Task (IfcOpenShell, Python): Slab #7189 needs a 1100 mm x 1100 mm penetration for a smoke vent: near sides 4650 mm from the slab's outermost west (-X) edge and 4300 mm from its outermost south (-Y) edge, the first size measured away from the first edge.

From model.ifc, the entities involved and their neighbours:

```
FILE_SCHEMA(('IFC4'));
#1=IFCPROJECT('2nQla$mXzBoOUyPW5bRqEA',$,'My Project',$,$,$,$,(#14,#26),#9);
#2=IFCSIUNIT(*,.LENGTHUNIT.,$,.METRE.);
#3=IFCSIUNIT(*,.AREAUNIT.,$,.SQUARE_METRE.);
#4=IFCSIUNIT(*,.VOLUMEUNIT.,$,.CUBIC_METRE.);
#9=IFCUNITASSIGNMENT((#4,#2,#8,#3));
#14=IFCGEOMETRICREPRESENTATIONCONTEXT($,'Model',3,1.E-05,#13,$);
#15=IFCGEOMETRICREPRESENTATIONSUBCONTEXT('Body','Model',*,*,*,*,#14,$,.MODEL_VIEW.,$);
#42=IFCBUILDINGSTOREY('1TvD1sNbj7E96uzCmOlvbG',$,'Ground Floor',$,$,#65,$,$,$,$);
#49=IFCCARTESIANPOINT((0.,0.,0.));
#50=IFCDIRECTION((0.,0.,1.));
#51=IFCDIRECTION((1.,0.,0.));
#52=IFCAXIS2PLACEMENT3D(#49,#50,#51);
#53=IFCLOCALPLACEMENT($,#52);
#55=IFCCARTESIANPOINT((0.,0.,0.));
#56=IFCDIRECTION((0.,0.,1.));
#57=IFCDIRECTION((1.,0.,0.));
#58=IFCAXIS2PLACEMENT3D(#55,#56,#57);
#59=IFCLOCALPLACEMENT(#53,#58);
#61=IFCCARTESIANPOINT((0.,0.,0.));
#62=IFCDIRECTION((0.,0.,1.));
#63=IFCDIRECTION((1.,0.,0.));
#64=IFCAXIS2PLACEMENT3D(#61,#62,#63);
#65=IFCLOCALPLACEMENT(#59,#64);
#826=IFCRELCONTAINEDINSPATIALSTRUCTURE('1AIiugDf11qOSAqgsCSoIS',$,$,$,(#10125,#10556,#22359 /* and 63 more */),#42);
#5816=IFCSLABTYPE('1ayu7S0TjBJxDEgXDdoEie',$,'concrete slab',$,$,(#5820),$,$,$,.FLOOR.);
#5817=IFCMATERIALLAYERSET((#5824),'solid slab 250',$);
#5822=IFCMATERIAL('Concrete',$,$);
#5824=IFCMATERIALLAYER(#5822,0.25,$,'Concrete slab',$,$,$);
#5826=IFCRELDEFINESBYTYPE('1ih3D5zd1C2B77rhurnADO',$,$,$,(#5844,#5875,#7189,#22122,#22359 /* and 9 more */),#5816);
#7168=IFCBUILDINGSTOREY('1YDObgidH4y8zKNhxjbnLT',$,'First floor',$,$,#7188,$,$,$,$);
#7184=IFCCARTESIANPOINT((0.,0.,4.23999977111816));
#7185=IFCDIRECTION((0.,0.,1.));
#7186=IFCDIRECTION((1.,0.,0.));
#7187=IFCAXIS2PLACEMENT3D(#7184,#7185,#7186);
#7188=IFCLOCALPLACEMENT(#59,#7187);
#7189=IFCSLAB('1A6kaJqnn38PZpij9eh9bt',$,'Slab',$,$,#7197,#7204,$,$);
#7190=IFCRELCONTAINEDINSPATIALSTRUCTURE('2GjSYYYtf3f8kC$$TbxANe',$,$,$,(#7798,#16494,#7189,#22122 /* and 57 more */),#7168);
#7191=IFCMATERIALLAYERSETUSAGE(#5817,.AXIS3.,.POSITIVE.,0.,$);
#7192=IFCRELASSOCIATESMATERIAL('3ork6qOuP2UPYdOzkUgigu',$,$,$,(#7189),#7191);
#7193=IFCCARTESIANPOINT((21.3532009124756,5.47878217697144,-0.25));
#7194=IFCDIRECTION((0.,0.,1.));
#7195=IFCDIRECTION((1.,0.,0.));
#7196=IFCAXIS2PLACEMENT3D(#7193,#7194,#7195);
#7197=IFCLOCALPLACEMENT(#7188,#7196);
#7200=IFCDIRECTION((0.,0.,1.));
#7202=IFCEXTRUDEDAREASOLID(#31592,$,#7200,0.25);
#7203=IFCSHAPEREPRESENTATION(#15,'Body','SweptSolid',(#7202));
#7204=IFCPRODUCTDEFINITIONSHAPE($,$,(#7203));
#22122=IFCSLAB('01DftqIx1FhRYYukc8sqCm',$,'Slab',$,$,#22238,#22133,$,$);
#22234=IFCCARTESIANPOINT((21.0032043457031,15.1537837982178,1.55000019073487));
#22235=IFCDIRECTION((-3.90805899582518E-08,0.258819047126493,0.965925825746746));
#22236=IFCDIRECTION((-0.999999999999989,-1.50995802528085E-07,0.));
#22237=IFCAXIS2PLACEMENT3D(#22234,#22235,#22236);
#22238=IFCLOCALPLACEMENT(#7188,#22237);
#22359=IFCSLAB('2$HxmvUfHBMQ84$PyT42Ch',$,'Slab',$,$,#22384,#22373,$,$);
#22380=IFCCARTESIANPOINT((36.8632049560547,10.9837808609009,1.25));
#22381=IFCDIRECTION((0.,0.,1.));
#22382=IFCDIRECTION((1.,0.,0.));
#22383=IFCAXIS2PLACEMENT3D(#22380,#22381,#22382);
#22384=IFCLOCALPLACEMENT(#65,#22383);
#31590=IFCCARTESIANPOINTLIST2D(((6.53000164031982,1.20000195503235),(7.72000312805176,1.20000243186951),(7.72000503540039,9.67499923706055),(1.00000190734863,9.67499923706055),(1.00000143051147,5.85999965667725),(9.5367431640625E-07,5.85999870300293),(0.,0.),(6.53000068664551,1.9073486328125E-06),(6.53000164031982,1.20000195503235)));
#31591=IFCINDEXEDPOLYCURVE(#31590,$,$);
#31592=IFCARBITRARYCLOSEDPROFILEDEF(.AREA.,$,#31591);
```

```python
import numpy as np
import ifcopenshell
import ifcopenshell.api.feature
import ifcopenshell.api.geometry
import ifcopenshell.api.root
import ifcopenshell.geom
import ifcopenshell.util.placement
import ifcopenshell.util.representation
import ifcopenshell.util.shape
import ifcopenshell.util.unit

model = ifcopenshell.open("model.ifc")
unit_scale = ifcopenshell.util.unit.calculate_unit_scale(model)
settings = ifcopenshell.geom.settings()


def volume(element):
    """Net volume in cubic metres, openings subtracted."""
    shape = ifcopenshell.geom.create_shape(settings, element)
    return ifcopenshell.util.shape.get_volume(shape.geometry)


slab = model.by_id(7189)
before = volume(slab)

# Extent in the slab's own axes, in metres. The edges named are its -X and -Y sides.
slab_shape = ifcopenshell.geom.create_shape(settings, slab)
vertices = ifcopenshell.util.shape.get_vertices(slab_shape.geometry)
x_min, y_min, bottom = vertices.min(axis=0)
top = vertices[:, 2].max()

opening = ifcopenshell.api.root.create_entity(model, ifc_class="IfcOpeningElement", name="Smoke vent opening", predefined_type="OPENING")
context = ifcopenshell.util.representation.get_context(model, "Model", "Body", "MODEL_VIEW")
width, depth = 1.1, 1.1
outline = [(0.0, 0.0), (width, 0.0), (width, depth), (0.0, depth), (0.0, 0.0)]
# Overshoot both faces by 50 mm so the cut is clean.
shape = ifcopenshell.api.geometry.add_slab_representation(
    model, context=context, depth=top - bottom + 0.1, polyline=outline
)
ifcopenshell.api.geometry.assign_representation(model, product=opening, representation=shape)

matrix = ifcopenshell.util.placement.get_local_placement(slab.ObjectPlacement)
matrix[:, 3] = matrix @ np.append(np.array([x_min + 4.65, y_min + 4.3, bottom - 0.05]) / unit_scale, 1.0)
ifcopenshell.api.geometry.edit_object_placement(model, product=opening, matrix=matrix, is_si=False)
ifcopenshell.api.feature.add_feature(model, feature=opening, element=slab)

after = volume(slab)

print(f"slab volume {before:.3f} -> {after:.3f} m3")

model.write("model_edited.ifc")
```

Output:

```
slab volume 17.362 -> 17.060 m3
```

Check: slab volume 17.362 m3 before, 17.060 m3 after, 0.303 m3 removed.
